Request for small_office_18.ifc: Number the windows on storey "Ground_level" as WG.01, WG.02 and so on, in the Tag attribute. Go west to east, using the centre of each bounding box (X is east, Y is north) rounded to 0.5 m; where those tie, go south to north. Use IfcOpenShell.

First a look at what the model holds.

```python
import ifcopenshell
import ifcopenshell.util.element
import ifcopenshell.util.placement

model = ifcopenshell.open("small_office_18.ifc")
print(model.schema)
storey = next(s for s in model.by_type("IfcBuildingStorey") if s.Name == "Ground_level")
windows = [e for e in ifcopenshell.util.element.get_decomposition(storey) if e.is_a("IfcWindow")]
for e in sorted(windows, key=lambda e: e.id()):
    origin = ifcopenshell.util.placement.get_local_placement(e.ObjectPlacement)[:3, 3]
    print(e.id(), e.Tag, e.Name, origin.round(2) + 0.0, sep=" | ")
```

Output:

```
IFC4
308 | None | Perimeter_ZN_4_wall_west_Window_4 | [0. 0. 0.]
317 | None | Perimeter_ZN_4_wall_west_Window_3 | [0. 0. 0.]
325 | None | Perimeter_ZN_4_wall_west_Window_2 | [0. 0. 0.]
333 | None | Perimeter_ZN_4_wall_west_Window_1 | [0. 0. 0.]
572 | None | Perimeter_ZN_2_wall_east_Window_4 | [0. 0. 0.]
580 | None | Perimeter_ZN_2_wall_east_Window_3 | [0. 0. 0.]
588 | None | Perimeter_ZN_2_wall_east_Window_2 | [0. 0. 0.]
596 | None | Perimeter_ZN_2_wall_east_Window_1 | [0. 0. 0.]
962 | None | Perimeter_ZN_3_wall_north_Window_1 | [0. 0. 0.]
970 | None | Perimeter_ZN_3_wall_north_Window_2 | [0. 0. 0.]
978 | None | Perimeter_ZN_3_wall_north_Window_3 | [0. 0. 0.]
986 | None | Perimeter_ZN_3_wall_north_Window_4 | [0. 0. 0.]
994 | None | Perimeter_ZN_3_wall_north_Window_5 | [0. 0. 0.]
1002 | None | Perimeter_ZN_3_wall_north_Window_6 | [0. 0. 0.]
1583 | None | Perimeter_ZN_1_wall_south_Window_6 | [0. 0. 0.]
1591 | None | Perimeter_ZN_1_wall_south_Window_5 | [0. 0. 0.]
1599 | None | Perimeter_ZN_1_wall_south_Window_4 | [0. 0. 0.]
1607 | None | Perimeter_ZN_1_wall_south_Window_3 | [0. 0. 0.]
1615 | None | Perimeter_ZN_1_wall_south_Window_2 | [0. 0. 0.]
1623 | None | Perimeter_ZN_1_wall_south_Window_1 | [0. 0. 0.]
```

```python
import ifcopenshell
import ifcopenshell.geom
import ifcopenshell.util.element
import ifcopenshell.util.shape

model = ifcopenshell.open("small_office_18.ifc")
settings = ifcopenshell.geom.settings()
settings.set("use-world-coords", True)


def centre(element):
    shape = ifcopenshell.geom.create_shape(settings, element)
    return ifcopenshell.util.shape.get_bbox_centroid(shape.geometry)


storey = next(s for s in model.by_type("IfcBuildingStorey") if s.Name == "Ground_level")
windows = [e for e in ifcopenshell.util.element.get_decomposition(storey) if e.is_a("IfcWindow")]

# Insertion points can sit at a corner or the storey origin, so sort by the geometry (in metres).
centres = {e: centre(e) for e in windows}
windows.sort(key=lambda e: (round(centres[e][0] / 0.5), centres[e][1]))

for i, e in enumerate(windows, start=1):
    number = f"WG.{i:02d}"
    e.Tag = number
    print(e.id(), number)

model.write("small_office_18_edited.ifc")
```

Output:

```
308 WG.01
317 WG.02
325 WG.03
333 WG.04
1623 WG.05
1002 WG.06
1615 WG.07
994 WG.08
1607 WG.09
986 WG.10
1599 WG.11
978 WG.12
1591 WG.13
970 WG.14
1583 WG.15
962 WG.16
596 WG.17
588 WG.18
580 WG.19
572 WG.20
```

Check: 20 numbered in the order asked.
